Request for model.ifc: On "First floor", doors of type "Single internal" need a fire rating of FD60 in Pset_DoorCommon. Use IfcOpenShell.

First a look at what the model holds.

```python
import ifcopenshell
import ifcopenshell.util.element

model = ifcopenshell.open("model.ifc")
print(model.schema)
storey = next(s for s in model.by_type("IfcBuildingStorey") if s.Name == "First floor")
doors = [e for e in ifcopenshell.util.element.get_decomposition(storey) if e.is_a("IfcDoor")]
seen = {}
for e in doors:
    element_type = ifcopenshell.util.element.get_type(e)
    key = (element_type.Name if element_type != e and element_type else None, ifcopenshell.util.element.get_pset(e, "Pset_DoorCommon", "FireRating"))
    seen[key] = seen.get(key, 0) + 1
for (name, value), count in sorted(seen.items(), key=str):
    print(count, "x", name, "|", value)
```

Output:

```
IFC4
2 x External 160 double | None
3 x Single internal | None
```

```python
import ifcopenshell
import ifcopenshell.api.pset
import ifcopenshell.util.element

model = ifcopenshell.open("model.ifc")

storey = next(s for s in model.by_type("IfcBuildingStorey") if s.Name == "First floor")
doors = [e for e in ifcopenshell.util.element.get_decomposition(storey) if e.is_a("IfcDoor")]

count = 0
for e in doors:
    element_type = ifcopenshell.util.element.get_type(e)
    if element_type in (None, e) or element_type.Name != "Single internal":
        continue
    # add_pset returns the element's existing set when there is one.
    pset = ifcopenshell.api.pset.add_pset(model, product=e, name="Pset_DoorCommon")
    ifcopenshell.api.pset.edit_pset(model, pset=pset, properties={"FireRating": "FD60"})
    count += 1

print(count, "doors updated")

model.write("model_edited.ifc")
```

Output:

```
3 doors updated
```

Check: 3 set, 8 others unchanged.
